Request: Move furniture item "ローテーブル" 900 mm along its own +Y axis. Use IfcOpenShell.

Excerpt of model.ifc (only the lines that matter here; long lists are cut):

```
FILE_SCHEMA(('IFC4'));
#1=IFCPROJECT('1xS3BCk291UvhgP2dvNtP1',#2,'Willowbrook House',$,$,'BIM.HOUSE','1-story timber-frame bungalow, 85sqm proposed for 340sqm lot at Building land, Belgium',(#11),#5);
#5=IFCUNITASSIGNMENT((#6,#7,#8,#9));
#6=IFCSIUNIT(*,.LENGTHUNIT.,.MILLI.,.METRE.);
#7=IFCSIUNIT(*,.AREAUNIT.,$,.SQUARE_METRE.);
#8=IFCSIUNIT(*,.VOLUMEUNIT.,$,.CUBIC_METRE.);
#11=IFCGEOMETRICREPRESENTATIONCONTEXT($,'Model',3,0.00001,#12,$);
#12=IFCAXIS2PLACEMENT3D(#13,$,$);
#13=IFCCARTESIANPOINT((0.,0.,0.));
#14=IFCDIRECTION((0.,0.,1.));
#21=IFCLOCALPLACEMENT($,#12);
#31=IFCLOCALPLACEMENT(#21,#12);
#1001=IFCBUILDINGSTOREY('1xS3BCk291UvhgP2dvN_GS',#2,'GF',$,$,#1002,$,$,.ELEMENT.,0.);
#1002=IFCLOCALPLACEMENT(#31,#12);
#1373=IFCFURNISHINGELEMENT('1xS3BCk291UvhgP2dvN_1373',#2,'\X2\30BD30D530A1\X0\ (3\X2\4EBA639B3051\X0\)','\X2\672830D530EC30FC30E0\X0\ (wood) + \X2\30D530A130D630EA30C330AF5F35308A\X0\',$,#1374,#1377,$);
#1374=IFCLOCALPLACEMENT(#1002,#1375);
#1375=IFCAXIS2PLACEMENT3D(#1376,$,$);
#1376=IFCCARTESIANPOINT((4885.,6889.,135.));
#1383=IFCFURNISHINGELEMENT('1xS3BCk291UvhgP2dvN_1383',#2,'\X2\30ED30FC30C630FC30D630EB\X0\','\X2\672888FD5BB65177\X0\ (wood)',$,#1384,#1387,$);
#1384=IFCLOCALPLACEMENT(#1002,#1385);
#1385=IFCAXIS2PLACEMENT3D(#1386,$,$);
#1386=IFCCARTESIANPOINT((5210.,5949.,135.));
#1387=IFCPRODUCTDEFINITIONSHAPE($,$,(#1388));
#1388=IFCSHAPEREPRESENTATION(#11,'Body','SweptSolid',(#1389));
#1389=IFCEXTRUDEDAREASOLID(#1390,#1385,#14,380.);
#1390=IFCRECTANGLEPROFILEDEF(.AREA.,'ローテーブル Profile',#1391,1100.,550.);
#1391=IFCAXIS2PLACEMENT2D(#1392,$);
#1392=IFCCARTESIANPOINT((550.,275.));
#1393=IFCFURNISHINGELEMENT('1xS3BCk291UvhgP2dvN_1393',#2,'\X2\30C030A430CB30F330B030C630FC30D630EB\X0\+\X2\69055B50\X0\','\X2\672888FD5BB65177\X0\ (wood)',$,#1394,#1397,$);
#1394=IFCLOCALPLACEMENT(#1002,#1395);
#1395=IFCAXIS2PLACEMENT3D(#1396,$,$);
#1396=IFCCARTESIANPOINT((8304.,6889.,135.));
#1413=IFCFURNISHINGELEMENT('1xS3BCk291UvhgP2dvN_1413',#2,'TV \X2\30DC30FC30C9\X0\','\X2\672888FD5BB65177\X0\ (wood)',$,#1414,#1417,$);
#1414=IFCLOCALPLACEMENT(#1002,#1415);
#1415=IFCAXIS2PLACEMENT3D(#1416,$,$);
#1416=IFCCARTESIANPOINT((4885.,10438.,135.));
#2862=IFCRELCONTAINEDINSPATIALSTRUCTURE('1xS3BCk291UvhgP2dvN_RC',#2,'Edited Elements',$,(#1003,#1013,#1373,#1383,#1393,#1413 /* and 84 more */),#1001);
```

```python
import ifcopenshell
import ifcopenshell.api.geometry
import ifcopenshell.util.placement

model = ifcopenshell.open("model.ifc")

item = model.by_guid("1xS3BCk291UvhgP2dvN_1383")
matrix = ifcopenshell.util.placement.get_local_placement(item.ObjectPlacement)
matrix[:3, 3] += matrix[:3, 1] * 900.0
ifcopenshell.api.geometry.edit_object_placement(model, product=item, matrix=matrix, is_si=False)

print(ifcopenshell.util.placement.get_local_placement(item.ObjectPlacement).round(3) + 0.0)

model.write("model_v2.ifc")
```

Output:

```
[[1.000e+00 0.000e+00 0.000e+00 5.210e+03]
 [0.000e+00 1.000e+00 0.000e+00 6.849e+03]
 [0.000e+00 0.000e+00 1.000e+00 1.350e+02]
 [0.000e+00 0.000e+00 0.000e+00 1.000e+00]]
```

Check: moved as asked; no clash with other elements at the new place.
